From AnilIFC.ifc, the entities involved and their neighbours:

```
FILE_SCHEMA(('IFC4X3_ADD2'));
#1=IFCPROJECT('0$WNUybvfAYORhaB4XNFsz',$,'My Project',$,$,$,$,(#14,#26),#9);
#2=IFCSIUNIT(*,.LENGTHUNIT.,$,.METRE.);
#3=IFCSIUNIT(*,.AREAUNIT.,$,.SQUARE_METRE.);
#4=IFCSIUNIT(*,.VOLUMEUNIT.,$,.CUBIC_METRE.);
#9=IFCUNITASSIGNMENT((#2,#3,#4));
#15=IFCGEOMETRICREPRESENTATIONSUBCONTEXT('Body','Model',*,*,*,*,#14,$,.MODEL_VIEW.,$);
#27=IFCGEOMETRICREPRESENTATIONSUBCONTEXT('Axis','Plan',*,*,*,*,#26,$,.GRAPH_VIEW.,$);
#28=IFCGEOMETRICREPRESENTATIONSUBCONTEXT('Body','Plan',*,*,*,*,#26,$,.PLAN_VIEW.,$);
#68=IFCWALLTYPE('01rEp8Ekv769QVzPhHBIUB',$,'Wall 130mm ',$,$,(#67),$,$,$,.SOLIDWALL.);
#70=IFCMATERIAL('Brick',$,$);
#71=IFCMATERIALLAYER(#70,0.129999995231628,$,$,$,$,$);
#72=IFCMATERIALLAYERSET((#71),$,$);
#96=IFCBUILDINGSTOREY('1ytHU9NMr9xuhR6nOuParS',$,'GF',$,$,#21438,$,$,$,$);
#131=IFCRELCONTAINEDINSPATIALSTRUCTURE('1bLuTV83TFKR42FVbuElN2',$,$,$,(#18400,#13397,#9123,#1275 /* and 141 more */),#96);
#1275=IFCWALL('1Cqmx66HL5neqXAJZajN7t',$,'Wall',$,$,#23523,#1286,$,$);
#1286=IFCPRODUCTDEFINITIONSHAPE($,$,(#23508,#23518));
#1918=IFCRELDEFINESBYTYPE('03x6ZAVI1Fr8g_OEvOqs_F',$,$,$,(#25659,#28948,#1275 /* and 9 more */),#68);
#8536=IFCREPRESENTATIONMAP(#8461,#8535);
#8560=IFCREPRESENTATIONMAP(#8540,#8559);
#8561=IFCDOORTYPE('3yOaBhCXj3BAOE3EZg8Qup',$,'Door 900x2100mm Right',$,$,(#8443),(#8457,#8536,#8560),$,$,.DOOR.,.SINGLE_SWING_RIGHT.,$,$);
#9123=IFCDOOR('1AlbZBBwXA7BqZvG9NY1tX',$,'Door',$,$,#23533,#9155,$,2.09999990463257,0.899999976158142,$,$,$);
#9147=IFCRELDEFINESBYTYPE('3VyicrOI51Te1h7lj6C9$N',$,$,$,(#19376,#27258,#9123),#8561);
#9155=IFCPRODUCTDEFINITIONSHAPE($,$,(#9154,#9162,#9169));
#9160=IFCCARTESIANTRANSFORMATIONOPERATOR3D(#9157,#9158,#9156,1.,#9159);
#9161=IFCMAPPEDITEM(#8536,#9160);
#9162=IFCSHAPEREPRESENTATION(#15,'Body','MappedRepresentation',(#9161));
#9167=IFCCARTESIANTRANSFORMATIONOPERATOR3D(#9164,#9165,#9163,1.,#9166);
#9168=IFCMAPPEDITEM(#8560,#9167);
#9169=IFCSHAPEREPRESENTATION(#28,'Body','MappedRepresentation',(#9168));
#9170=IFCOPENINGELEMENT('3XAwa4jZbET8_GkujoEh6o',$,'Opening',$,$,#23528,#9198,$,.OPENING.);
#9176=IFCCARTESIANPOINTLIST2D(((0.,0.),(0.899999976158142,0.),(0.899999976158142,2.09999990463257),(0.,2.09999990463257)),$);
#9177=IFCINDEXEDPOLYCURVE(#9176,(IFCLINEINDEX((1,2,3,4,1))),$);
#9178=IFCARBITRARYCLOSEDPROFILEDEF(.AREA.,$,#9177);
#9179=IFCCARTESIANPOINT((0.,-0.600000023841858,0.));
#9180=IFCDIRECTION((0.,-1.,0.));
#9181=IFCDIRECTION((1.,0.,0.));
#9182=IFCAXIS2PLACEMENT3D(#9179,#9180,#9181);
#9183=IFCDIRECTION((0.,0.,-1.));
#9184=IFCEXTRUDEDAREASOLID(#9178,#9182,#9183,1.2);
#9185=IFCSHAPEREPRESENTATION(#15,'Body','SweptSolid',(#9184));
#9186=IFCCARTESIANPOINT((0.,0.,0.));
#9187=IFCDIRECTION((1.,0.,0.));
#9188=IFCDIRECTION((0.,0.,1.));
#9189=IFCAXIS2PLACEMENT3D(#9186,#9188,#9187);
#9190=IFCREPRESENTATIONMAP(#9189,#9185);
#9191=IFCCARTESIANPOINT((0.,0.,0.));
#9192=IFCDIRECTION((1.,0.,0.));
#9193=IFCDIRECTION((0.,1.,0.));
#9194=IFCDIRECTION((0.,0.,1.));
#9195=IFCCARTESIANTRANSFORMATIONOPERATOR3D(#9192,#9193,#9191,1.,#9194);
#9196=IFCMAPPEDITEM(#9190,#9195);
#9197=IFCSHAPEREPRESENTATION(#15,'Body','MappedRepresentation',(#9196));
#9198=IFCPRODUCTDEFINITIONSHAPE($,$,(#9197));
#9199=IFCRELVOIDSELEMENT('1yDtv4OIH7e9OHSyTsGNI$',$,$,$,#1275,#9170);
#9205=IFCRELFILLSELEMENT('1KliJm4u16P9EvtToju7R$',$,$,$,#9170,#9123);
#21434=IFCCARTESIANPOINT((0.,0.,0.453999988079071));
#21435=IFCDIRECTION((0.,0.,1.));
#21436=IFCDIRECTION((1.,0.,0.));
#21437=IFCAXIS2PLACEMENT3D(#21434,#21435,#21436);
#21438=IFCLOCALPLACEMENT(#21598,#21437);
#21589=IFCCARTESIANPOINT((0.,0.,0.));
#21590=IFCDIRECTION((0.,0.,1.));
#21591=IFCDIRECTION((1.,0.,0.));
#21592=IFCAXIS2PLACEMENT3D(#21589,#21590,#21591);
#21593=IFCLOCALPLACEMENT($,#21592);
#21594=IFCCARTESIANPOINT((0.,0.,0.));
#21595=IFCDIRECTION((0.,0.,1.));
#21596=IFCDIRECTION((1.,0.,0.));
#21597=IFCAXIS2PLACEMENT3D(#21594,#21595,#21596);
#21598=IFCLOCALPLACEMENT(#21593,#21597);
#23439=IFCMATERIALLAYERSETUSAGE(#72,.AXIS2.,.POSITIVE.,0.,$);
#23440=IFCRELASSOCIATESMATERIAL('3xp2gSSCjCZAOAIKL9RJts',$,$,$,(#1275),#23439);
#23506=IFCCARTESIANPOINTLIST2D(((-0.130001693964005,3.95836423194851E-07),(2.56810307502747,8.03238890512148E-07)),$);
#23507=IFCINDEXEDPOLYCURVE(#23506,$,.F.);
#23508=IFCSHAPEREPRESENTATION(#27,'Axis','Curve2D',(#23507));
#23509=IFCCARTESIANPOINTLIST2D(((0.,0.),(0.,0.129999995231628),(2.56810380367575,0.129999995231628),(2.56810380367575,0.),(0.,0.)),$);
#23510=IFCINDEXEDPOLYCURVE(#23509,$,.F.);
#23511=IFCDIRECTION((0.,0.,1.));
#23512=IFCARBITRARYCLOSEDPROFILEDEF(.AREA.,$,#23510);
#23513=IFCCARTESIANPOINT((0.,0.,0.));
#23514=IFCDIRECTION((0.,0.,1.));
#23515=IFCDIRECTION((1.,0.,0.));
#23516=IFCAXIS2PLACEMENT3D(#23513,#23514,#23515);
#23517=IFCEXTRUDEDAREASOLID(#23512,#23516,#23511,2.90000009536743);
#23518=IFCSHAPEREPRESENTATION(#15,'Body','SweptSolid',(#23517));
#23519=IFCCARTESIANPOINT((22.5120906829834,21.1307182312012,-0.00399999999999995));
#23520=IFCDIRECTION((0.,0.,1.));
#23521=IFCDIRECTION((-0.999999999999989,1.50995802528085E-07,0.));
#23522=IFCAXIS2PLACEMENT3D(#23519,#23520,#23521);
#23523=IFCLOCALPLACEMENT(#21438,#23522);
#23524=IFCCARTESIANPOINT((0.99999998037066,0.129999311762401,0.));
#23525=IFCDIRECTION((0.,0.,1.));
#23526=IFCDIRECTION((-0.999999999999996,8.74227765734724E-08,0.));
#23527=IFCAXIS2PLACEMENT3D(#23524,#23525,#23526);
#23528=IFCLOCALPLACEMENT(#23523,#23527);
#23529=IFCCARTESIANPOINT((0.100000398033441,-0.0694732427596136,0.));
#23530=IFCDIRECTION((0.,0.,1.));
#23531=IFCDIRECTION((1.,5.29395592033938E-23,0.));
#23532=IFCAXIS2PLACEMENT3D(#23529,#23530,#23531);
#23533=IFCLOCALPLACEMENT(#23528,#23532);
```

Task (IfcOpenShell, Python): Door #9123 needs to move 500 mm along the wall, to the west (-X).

```python
import ifcopenshell
import ifcopenshell.api.geometry
import ifcopenshell.util.placement

model = ifcopenshell.open("AnilIFC.ifc")

door = model.by_guid("1AlbZBBwXA7BqZvG9NY1tX")
opening = door.FillsVoids[0].RelatingOpeningElement
wall = opening.VoidsElements[0].RelatingBuildingElement

wall_matrix = ifcopenshell.util.placement.get_local_placement(wall.ObjectPlacement)
shift = wall_matrix[:3, 0] * 0.5
before = ifcopenshell.util.placement.get_local_placement(door.ObjectPlacement)[:3, 3].copy()

# The door is placed relative to its opening, so it follows when the opening moves.
matrix = ifcopenshell.util.placement.get_local_placement(opening.ObjectPlacement)
matrix[:3, 3] += shift
ifcopenshell.api.geometry.edit_object_placement(
    model, product=opening, matrix=matrix, is_si=False, should_transform_children=True
)

after = ifcopenshell.util.placement.get_local_placement(door.ObjectPlacement)[:3, 3]
print("door moved by", (after - before).round(3) + 0.0)

model.write("AnilIFC_v2.ifc")
```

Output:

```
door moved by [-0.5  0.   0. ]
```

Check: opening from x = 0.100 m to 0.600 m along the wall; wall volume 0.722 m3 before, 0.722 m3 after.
